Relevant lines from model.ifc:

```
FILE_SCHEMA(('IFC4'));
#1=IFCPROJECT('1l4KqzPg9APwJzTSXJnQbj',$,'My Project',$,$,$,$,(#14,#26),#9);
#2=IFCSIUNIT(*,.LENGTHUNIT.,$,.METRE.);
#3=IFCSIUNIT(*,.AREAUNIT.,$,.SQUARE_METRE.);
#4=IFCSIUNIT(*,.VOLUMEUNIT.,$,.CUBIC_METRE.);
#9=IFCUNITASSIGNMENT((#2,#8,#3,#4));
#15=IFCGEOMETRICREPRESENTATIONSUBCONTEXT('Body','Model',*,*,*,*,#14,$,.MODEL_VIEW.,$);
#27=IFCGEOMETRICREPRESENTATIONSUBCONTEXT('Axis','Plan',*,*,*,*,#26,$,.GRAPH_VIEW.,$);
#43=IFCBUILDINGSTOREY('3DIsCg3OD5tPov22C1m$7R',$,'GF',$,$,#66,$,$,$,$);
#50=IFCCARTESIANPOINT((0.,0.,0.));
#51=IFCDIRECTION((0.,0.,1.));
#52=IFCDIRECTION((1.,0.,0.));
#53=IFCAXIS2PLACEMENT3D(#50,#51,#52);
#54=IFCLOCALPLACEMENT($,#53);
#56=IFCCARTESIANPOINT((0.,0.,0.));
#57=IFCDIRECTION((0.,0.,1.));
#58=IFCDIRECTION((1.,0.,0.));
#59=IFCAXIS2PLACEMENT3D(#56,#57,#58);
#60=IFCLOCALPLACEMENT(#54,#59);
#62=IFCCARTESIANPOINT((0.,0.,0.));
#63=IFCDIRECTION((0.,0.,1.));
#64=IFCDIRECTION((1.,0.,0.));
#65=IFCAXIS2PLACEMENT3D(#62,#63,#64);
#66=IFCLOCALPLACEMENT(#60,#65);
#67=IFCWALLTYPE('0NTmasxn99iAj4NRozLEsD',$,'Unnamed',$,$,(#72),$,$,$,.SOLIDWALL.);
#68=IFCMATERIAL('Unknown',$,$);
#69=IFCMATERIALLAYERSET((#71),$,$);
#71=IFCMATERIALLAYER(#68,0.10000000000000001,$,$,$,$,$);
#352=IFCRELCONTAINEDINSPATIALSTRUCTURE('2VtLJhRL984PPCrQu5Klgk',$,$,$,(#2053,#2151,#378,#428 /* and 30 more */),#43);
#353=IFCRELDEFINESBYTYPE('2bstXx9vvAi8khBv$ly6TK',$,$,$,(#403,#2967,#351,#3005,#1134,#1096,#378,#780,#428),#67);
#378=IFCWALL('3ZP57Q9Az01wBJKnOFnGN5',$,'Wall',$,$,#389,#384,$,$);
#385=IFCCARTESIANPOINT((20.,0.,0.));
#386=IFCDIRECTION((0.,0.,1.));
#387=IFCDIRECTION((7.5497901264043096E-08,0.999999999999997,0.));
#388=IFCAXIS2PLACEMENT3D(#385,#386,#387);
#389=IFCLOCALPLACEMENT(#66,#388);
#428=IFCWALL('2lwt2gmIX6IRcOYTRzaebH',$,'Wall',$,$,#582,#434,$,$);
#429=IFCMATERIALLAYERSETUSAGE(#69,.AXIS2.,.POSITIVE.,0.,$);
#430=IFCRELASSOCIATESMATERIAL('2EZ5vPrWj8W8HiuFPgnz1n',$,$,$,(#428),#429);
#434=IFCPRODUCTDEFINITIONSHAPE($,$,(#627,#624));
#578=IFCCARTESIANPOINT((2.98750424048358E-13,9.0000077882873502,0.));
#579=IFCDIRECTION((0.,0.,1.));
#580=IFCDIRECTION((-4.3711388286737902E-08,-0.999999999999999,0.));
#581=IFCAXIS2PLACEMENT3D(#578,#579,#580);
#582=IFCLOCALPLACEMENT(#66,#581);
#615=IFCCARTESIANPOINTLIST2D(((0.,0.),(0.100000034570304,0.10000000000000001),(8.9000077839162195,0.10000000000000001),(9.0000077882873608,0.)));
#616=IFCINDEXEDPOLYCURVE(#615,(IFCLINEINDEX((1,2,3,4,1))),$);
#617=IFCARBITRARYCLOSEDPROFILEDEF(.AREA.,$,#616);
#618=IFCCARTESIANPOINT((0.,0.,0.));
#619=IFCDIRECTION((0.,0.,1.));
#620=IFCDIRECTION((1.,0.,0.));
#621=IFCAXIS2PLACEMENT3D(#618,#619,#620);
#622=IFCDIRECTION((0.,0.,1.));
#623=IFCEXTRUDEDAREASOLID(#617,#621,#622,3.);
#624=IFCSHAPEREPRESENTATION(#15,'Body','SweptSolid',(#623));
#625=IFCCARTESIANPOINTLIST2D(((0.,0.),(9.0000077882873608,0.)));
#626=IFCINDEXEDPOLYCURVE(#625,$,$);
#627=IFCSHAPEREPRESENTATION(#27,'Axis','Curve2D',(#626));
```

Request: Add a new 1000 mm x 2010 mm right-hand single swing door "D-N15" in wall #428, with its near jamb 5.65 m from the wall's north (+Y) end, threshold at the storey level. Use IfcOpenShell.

```python
import numpy as np
import ifcopenshell
import ifcopenshell.api.feature
import ifcopenshell.api.geometry
import ifcopenshell.api.root
import ifcopenshell.api.spatial
import ifcopenshell.geom
import ifcopenshell.util.element
import ifcopenshell.util.placement
import ifcopenshell.util.representation
import ifcopenshell.util.shape
import ifcopenshell.util.unit

model = ifcopenshell.open("model.ifc")
unit_scale = ifcopenshell.util.unit.calculate_unit_scale(model)
settings = ifcopenshell.geom.settings()


def volume(element):
    """Net volume in cubic metres, openings subtracted."""
    shape = ifcopenshell.geom.create_shape(settings, element)
    return ifcopenshell.util.shape.get_volume(shape.geometry)


wall = model.by_guid("2lwt2gmIX6IRcOYTRzaebH")
storey = ifcopenshell.util.element.get_container(wall, ifc_class="IfcBuildingStorey")
context = ifcopenshell.util.representation.get_context(model, "Model", "Body", "MODEL_VIEW")
before = volume(wall)

width, height, from_end, sill = 1, 2.01, 5.65, 0.0  # metres

# The wall runs along its own X axis, and the end named is its -X end.
wall_shape = ifcopenshell.geom.create_shape(settings, wall)
x, y, z = ifcopenshell.util.shape.get_vertices(wall_shape.geometry).T
start = x.min() + from_end
face, thickness = float(y.min()), float(y.max() - y.min())
wall_matrix = ifcopenshell.util.placement.get_local_placement(wall.ObjectPlacement)
level = ifcopenshell.util.placement.get_local_placement(storey.ObjectPlacement)[2, 3]


def in_wall(x, y):
    """Placement at x, y metres in the wall's axes, at sill height."""
    matrix = wall_matrix.copy()
    matrix[:, 3] = wall_matrix @ np.array([x / unit_scale, y / unit_scale, 0.0, 1.0])
    matrix[2, 3] = level + sill / unit_scale
    return matrix


# Opening: a box that overshoots both wall faces by 50 mm.
opening = ifcopenshell.api.root.create_entity(model, ifc_class="IfcOpeningElement", predefined_type="OPENING")
box = ifcopenshell.api.geometry.add_wall_representation(
    model, context=context, length=width, height=height, thickness=thickness + 0.1
)
ifcopenshell.api.geometry.assign_representation(model, product=opening, representation=box)
ifcopenshell.api.geometry.edit_object_placement(model, product=opening, matrix=in_wall(start, face - 0.05), is_si=False)
ifcopenshell.api.feature.add_feature(model, feature=opening, element=wall)

door = ifcopenshell.api.root.create_entity(model, ifc_class="IfcDoor", name="D-N15", predefined_type="DOOR")
door.OverallWidth, door.OverallHeight = width / unit_scale, height / unit_scale
door.OperationType = "SINGLE_SWING_RIGHT"
body = ifcopenshell.api.geometry.add_door_representation(
    model,
    context=context,
    overall_width=door.OverallWidth,
    overall_height=door.OverallHeight,
    operation_type="SINGLE_SWING_RIGHT",
    lining_properties={"LiningDepth": thickness / unit_scale, "ThresholdDepth": thickness / unit_scale},
)
ifcopenshell.api.geometry.assign_representation(model, product=door, representation=body)
ifcopenshell.api.spatial.assign_container(model, products=[door], relating_structure=storey)
ifcopenshell.api.feature.add_filling(model, opening=opening, element=door)

# The lining spans the wall, so the door starts at the wall face.
ifcopenshell.api.geometry.edit_object_placement(model, product=door, matrix=in_wall(start, face), is_si=False)

after = volume(wall)

print(f"wall volume {before:.3f} -> {after:.3f} m3")

model.write("model_rev.ifc")
```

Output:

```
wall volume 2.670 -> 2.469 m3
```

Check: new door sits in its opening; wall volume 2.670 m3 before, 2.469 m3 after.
